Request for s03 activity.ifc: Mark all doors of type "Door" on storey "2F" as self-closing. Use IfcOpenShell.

First a look at what the model holds.

```python
import ifcopenshell
import ifcopenshell.util.element

model = ifcopenshell.open("s03 activity.ifc")
print(model.schema)
storey = next(s for s in model.by_type("IfcBuildingStorey") if s.Name == "2F")
doors = [e for e in ifcopenshell.util.element.get_decomposition(storey) if e.is_a("IfcDoor")]
seen = {}
for e in doors:
    element_type = ifcopenshell.util.element.get_type(e)
    key = (element_type.Name if element_type != e and element_type else None, ifcopenshell.util.element.get_pset(e, "Pset_DoorCommon", "SelfClosing"))
    seen[key] = seen.get(key, 0) + 1
for (name, value), count in sorted(seen.items(), key=str):
    print(count, "x", name, "|", value)
```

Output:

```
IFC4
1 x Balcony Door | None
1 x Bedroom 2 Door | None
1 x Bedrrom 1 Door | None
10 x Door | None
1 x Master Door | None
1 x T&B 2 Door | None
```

```python
import ifcopenshell
import ifcopenshell.api.pset
import ifcopenshell.util.element

model = ifcopenshell.open("s03 activity.ifc")

storey = next(s for s in model.by_type("IfcBuildingStorey") if s.Name == "2F")
doors = [e for e in ifcopenshell.util.element.get_decomposition(storey) if e.is_a("IfcDoor")]

count = 0
for e in doors:
    element_type = ifcopenshell.util.element.get_type(e)
    if element_type in (None, e) or element_type.Name != "Door":
        continue
    # add_pset returns the element's existing set when there is one.
    pset = ifcopenshell.api.pset.add_pset(model, product=e, name="Pset_DoorCommon")
    ifcopenshell.api.pset.edit_pset(model, pset=pset, properties={"SelfClosing": True})
    count += 1

print(count, "doors updated")

model.write("s03 activity-out.ifc")
```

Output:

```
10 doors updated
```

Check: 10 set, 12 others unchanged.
